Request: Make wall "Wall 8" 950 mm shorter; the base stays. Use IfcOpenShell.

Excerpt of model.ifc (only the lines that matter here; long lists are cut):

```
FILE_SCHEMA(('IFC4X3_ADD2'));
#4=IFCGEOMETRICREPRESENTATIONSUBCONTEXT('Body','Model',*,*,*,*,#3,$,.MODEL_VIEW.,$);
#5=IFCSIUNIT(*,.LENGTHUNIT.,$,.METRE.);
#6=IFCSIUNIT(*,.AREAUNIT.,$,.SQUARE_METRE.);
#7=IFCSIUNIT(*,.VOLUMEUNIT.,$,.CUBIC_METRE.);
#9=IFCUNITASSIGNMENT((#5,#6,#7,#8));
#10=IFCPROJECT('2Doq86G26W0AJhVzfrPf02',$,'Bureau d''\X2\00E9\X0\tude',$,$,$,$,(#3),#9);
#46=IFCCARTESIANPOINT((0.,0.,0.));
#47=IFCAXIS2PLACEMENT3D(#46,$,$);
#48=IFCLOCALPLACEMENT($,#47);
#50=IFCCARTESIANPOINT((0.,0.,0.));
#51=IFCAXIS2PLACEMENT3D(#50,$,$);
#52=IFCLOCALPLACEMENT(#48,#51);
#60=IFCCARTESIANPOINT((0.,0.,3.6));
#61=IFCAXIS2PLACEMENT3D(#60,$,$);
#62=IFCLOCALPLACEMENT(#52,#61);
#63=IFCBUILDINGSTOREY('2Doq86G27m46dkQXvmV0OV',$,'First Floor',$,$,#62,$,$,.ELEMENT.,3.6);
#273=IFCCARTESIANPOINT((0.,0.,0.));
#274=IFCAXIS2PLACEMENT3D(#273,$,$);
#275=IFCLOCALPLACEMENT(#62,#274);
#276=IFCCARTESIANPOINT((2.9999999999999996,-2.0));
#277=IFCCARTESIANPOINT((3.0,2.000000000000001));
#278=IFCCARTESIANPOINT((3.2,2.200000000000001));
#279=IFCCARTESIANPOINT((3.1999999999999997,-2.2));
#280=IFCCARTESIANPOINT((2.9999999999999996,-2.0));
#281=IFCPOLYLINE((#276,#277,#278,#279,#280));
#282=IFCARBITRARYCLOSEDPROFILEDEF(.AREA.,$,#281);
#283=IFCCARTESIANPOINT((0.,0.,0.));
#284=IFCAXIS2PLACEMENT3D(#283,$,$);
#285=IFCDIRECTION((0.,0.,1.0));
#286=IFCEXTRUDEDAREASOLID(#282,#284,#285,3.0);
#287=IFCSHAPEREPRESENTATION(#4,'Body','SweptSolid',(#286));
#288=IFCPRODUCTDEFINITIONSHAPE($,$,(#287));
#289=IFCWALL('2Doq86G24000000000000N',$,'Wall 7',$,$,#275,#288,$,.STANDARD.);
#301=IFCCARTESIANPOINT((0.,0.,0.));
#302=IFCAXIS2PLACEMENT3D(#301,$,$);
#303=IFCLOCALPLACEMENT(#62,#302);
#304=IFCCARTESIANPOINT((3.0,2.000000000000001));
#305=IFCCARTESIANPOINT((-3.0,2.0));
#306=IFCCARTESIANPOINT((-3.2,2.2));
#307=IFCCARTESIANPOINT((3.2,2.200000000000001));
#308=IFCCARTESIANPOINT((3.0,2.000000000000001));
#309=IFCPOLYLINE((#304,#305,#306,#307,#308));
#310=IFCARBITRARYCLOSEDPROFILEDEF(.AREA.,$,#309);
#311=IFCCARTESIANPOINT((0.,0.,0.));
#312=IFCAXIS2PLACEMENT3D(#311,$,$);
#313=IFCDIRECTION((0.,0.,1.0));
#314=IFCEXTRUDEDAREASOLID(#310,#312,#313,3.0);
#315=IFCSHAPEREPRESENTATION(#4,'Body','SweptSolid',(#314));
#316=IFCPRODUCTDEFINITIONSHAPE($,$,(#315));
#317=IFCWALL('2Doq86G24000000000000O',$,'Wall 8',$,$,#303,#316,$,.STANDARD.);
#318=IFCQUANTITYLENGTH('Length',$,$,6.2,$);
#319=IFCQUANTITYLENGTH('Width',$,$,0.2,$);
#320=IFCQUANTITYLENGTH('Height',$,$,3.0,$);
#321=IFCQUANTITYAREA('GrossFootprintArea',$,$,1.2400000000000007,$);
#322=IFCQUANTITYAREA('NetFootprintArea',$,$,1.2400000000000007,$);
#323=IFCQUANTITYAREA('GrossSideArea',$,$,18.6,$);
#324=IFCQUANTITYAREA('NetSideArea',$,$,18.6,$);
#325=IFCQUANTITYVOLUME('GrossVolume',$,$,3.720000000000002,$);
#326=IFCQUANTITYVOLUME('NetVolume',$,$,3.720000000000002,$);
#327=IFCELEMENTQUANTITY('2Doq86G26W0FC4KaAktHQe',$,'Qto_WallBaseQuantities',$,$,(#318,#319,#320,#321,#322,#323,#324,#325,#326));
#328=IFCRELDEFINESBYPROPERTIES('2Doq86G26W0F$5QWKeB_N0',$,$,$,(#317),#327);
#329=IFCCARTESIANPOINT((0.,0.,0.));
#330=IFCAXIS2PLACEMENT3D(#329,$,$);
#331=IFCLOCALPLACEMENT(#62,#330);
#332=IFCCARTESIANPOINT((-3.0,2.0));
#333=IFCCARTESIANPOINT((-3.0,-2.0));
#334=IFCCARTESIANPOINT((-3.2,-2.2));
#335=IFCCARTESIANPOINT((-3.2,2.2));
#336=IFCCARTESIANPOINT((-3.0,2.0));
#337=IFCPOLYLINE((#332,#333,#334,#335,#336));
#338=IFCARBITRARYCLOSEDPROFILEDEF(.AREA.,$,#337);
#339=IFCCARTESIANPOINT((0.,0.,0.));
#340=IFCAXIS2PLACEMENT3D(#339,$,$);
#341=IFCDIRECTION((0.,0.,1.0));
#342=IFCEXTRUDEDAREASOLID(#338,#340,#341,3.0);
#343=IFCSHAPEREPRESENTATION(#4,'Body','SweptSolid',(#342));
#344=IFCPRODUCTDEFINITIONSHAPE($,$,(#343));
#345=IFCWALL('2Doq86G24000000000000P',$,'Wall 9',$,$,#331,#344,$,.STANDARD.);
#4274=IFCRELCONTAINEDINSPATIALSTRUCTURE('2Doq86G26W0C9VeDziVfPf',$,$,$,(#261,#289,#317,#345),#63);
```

```python
import ifcopenshell
import ifcopenshell.api.pset
import ifcopenshell.geom
import ifcopenshell.util.element
import ifcopenshell.util.representation
import ifcopenshell.util.shape
import ifcopenshell.util.unit

model = ifcopenshell.open("model.ifc")
unit_scale = ifcopenshell.util.unit.calculate_unit_scale(model)
area_scale = ifcopenshell.util.unit.calculate_unit_scale(model, "AREAUNIT")
volume_scale = ifcopenshell.util.unit.calculate_unit_scale(model, "VOLUMEUNIT")
settings = ifcopenshell.geom.settings()


def volume(element):
    """Net volume in cubic metres, openings subtracted."""
    shape = ifcopenshell.geom.create_shape(settings, element)
    return ifcopenshell.util.shape.get_volume(shape.geometry)


wall = model.by_id(317)
before = volume(wall)

body = ifcopenshell.util.representation.get_representation(wall, "Model", "Body")
solid = body.Items[0]
old_height = solid.Depth
solid.Depth -= 0.95 / unit_scale
after = volume(wall)
thickness = 0.2  # wall thickness in metres

# Update the stored height, areas and volumes.
qto = model.by_id(ifcopenshell.util.element.get_pset(wall, "Qto_WallBaseQuantities", should_inherit=False)["id"])
ifcopenshell.api.pset.edit_qto(model, qto=qto, properties={
    "Height": solid.Depth,
    "GrossSideArea": ifcopenshell.util.element.get_pset(wall, "Qto_WallBaseQuantities", "GrossSideArea") * solid.Depth / old_height,
    "NetSideArea": after / thickness / area_scale,
    "GrossVolume": ifcopenshell.util.element.get_pset(wall, "Qto_WallBaseQuantities", "GrossVolume") * solid.Depth / old_height,
    "NetVolume": after / volume_scale,
})

print(f"height {old_height:g} -> {solid.Depth:g}, volume {before:.3f} -> {after:.3f} m3")

model.write("model_edited.ifc")
```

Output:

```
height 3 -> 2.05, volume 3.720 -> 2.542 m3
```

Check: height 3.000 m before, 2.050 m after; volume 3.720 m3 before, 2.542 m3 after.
